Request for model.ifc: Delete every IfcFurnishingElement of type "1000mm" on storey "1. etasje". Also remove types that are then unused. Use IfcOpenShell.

First a look at what the model holds.

```python
import ifcopenshell
import ifcopenshell.util.element

model = ifcopenshell.open("model.ifc")
print(model.schema)
storey = next(s for s in model.by_type("IfcBuildingStorey") if s.Name == "1. etasje")
furniture = [e for e in ifcopenshell.util.element.get_decomposition(storey) if e.is_a("IfcFurnishingElement")]
seen = {}
for e in furniture:
    element_type = ifcopenshell.util.element.get_type(e)
    name = element_type.Name if element_type not in (None, e) else None
    seen[name] = seen.get(name, 0) + 1
for name, count in sorted(seen.items(), key=str):
    print(count, "x", name)
```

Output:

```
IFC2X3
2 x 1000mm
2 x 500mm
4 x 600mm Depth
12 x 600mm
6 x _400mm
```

```python
import ifcopenshell
import ifcopenshell.api.root
import ifcopenshell.util.element

model = ifcopenshell.open("model.ifc")

storey = next(s for s in model.by_type("IfcBuildingStorey") if s.Name == "1. etasje")
furniture = [e for e in ifcopenshell.util.element.get_decomposition(storey) if e.is_a("IfcFurnishingElement")]
targets = [e for e in furniture if (t := ifcopenshell.util.element.get_type(e)) not in (None, e) and t.Name == "1000mm"]
types = {ifcopenshell.util.element.get_type(e) for e in targets} - {None, *targets}

for e in targets:
    ifcopenshell.api.root.remove_product(model, product=e)
print(len(targets), "removed")

unused = [t for t in types if not ifcopenshell.util.element.get_types(t)]
for t in unused:
    ifcopenshell.api.root.remove_product(model, product=t)
print(len(unused), "unused types removed")

model.write("model_v2.ifc")
```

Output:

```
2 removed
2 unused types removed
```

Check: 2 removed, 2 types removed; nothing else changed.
